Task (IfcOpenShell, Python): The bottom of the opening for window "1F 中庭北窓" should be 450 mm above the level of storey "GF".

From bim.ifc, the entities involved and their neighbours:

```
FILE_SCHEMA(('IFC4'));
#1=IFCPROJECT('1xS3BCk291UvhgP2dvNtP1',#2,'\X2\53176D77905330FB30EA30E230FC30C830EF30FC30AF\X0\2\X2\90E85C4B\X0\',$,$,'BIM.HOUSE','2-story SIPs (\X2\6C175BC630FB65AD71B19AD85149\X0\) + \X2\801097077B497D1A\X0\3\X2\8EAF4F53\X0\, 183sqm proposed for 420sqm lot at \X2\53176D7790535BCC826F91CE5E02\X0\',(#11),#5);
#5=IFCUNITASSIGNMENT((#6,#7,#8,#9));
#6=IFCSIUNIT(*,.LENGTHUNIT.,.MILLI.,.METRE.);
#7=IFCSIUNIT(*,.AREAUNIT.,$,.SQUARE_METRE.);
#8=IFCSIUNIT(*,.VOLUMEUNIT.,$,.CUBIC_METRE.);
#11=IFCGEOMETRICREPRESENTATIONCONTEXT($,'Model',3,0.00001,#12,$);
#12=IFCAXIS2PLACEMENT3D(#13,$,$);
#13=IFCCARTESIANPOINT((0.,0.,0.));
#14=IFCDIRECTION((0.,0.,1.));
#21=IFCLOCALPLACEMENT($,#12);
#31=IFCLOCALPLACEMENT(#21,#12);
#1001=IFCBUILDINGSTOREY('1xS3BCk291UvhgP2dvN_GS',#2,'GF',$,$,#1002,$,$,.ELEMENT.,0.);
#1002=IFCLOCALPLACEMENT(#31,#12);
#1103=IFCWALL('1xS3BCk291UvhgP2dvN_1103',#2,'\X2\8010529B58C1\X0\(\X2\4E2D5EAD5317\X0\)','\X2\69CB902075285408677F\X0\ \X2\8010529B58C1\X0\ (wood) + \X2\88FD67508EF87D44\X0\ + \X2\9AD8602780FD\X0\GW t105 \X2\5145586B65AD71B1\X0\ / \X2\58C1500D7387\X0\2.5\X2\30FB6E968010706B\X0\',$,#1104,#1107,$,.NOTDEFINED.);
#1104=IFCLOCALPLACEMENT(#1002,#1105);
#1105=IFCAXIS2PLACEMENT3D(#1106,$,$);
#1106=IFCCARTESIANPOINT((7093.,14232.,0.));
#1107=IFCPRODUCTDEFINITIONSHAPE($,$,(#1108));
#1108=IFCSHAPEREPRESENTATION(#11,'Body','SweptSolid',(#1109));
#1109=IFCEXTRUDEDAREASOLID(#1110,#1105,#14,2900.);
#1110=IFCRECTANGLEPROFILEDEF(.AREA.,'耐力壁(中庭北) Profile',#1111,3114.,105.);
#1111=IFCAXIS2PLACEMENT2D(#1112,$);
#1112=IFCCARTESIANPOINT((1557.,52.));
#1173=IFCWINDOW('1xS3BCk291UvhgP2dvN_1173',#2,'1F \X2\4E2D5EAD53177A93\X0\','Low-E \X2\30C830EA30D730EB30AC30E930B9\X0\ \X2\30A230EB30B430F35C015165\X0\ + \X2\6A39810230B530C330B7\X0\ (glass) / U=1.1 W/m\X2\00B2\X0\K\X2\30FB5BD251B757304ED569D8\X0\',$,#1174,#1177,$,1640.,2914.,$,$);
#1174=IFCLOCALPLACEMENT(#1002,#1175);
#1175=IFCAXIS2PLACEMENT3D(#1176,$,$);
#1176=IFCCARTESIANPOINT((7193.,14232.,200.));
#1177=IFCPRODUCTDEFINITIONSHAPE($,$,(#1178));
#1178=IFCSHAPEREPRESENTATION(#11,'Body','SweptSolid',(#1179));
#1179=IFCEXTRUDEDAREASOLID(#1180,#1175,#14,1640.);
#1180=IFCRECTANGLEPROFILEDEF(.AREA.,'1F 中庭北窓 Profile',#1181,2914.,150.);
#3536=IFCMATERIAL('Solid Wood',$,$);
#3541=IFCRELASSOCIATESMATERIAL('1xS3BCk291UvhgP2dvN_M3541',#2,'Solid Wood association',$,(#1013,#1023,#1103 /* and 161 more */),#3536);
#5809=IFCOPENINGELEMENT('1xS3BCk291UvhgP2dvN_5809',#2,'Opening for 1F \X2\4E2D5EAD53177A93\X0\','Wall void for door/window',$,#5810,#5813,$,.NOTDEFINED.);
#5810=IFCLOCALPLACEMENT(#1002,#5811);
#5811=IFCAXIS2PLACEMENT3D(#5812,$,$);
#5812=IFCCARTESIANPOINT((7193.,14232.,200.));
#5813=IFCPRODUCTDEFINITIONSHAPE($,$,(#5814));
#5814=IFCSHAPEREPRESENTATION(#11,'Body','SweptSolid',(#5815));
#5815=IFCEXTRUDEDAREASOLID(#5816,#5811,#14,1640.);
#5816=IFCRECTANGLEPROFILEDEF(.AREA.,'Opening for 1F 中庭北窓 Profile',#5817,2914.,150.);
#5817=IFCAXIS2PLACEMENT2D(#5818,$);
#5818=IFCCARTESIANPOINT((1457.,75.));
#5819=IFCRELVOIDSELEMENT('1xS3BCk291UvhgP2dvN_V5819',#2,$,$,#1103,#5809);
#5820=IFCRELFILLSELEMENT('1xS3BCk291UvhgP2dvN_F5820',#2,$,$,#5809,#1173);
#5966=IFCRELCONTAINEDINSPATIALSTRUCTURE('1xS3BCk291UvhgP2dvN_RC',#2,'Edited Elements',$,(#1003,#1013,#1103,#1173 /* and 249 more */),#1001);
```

```python
import numpy as np
import ifcopenshell
import ifcopenshell.api.geometry
import ifcopenshell.geom
import ifcopenshell.util.element
import ifcopenshell.util.placement
import ifcopenshell.util.shape
import ifcopenshell.util.unit

model = ifcopenshell.open("bim.ifc")
unit_scale = ifcopenshell.util.unit.calculate_unit_scale(model)

window = model.by_guid("1xS3BCk291UvhgP2dvN_1173")
opening = window.FillsVoids[0].RelatingOpeningElement
storey = ifcopenshell.util.element.get_container(window, ifc_class="IfcBuildingStorey")
level = ifcopenshell.util.placement.get_local_placement(storey.ObjectPlacement)[2, 3]

# The opening's origin need not be at the sill, so measure its lowest point.
shape = ifcopenshell.geom.create_shape(ifcopenshell.geom.settings(), opening)
bottom = ifcopenshell.util.shape.get_shape_bottom_elevation(shape, shape.geometry) / unit_scale
dz = level + 0.45 / unit_scale - bottom

shift = np.array([0.0, 0.0, dz])
# The window is not placed relative to its opening, so move both.
for product in (opening, window):
    matrix = ifcopenshell.util.placement.get_local_placement(product.ObjectPlacement)
    matrix[:3, 3] += shift
    ifcopenshell.api.geometry.edit_object_placement(model, product=product, matrix=matrix, is_si=False)

print(f"moved by {dz * unit_scale:+.3f} m")

model.write("bim-out.ifc")
```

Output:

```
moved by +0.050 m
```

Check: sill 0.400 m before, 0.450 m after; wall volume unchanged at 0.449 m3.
